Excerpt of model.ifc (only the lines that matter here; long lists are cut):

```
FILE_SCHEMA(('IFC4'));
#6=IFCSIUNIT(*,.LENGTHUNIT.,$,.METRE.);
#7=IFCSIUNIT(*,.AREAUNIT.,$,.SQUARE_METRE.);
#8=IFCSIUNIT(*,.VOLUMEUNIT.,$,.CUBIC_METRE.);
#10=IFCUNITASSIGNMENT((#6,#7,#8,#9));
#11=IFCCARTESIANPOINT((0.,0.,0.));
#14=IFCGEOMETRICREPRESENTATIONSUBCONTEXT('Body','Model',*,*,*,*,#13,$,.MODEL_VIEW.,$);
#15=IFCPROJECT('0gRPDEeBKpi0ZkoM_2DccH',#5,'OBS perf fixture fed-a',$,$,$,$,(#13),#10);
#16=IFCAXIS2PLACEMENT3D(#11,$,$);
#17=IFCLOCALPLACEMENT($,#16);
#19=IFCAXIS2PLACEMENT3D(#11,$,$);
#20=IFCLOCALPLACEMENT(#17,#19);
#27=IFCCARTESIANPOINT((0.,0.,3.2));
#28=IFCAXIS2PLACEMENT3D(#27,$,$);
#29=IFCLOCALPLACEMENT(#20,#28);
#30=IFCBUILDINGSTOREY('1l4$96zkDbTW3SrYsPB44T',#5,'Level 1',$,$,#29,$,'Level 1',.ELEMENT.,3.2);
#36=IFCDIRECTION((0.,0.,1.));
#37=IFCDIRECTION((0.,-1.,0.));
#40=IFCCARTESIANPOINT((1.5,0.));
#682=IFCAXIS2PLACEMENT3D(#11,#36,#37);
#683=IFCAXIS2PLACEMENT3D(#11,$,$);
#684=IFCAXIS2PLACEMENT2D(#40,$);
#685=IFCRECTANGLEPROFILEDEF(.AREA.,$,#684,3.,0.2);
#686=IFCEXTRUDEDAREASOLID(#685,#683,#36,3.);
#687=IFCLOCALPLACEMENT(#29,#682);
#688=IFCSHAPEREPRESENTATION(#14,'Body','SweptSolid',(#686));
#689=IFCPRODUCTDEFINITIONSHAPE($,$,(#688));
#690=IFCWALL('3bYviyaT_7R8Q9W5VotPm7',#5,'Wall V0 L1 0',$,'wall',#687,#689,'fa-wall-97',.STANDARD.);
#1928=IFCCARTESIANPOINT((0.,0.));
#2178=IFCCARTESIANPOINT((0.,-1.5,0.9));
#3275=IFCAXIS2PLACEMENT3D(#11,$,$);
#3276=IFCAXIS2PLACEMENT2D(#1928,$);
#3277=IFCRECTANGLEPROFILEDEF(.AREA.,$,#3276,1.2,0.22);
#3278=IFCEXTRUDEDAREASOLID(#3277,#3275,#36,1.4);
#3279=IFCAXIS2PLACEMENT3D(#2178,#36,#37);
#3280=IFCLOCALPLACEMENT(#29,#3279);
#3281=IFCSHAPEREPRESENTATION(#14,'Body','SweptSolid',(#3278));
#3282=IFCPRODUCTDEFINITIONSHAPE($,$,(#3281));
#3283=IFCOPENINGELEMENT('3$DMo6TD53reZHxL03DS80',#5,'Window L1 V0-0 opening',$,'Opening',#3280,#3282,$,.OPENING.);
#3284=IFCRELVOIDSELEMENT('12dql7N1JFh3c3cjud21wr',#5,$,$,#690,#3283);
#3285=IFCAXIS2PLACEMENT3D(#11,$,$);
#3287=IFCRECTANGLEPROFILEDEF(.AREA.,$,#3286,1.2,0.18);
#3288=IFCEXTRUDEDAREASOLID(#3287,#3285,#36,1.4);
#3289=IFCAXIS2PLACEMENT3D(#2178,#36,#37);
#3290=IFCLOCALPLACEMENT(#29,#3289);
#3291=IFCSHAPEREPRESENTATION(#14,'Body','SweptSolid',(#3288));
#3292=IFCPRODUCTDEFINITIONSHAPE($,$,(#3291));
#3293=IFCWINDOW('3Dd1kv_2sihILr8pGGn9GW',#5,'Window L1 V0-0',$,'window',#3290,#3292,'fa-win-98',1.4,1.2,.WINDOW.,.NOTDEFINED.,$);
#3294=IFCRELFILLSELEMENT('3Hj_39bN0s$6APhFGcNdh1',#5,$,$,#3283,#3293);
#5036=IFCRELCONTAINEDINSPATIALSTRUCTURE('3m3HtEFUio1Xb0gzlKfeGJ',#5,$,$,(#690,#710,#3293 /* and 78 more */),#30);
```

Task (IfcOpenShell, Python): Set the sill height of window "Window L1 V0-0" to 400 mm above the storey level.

```python
import numpy as np
import ifcopenshell
import ifcopenshell.api.geometry
import ifcopenshell.geom
import ifcopenshell.util.element
import ifcopenshell.util.placement
import ifcopenshell.util.shape
import ifcopenshell.util.unit

model = ifcopenshell.open("model.ifc")
unit_scale = ifcopenshell.util.unit.calculate_unit_scale(model)

window = model.by_guid("3Dd1kv_2sihILr8pGGn9GW")
opening = window.FillsVoids[0].RelatingOpeningElement
storey = ifcopenshell.util.element.get_container(window, ifc_class="IfcBuildingStorey")
level = ifcopenshell.util.placement.get_local_placement(storey.ObjectPlacement)[2, 3]

# The opening's origin need not be at the sill, so measure its lowest point.
shape = ifcopenshell.geom.create_shape(ifcopenshell.geom.settings(), opening)
bottom = ifcopenshell.util.shape.get_shape_bottom_elevation(shape, shape.geometry) / unit_scale
dz = level + 0.4 - bottom

shift = np.array([0.0, 0.0, dz])
# The window is not placed relative to its opening, so move both.
for product in (opening, window):
    matrix = ifcopenshell.util.placement.get_local_placement(product.ObjectPlacement)
    matrix[:3, 3] += shift
    ifcopenshell.api.geometry.edit_object_placement(model, product=product, matrix=matrix, is_si=False)

print(f"moved by {dz * unit_scale:+.3f} m")

model.write("model-out.ifc")
```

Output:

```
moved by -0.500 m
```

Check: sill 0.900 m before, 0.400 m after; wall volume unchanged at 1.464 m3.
